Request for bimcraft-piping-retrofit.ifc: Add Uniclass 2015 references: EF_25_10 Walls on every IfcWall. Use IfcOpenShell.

First a look at what the model holds.

```python
import ifcopenshell

model = ifcopenshell.open("bimcraft-piping-retrofit.ifc")
print(model.schema)
print("classifications:", [c.Name for c in model.by_type("IfcClassification")])
for ifc_class in ("IfcDoor", "IfcRoof", "IfcStair", "IfcWall", "IfcWindow"):
    print(ifc_class, len(model.by_type(ifc_class)))
```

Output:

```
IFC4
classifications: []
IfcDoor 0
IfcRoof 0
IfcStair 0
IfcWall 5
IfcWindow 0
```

```python
import ifcopenshell
import ifcopenshell.api.classification

model = ifcopenshell.open("bimcraft-piping-retrofit.ifc")

system = ifcopenshell.api.classification.add_classification(model, classification="Uniclass 2015")

codes = {
    "IfcWall": ("EF_25_10", "Walls"),
}
for ifc_class, (code, name) in codes.items():
    products = model.by_type(ifc_class)
    ifcopenshell.api.classification.add_reference(
        model, products=products, classification=system, identification=code, name=name
    )
    print(code, len(products))

model.write("bimcraft-piping-retrofit_v2.ifc")
```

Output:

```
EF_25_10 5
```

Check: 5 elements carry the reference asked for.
